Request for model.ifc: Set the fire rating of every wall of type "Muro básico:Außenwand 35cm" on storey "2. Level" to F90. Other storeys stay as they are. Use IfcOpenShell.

First a look at what the model holds.

```python
import ifcopenshell
import ifcopenshell.util.element

model = ifcopenshell.open("model.ifc")
print(model.schema)
storey = next(s for s in model.by_type("IfcBuildingStorey") if s.Name == "2. Level")
walls = [e for e in ifcopenshell.util.element.get_decomposition(storey) if e.is_a("IfcWall")]
seen = {}
for e in walls:
    element_type = ifcopenshell.util.element.get_type(e)
    key = (element_type.Name if element_type != e and element_type else None, ifcopenshell.util.element.get_pset(e, "Pset_WallCommon", "FireRating"))
    seen[key] = seen.get(key, 0) + 1
for (name, value), count in sorted(seen.items(), key=str):
    print(count, "x", name, "|", value)
```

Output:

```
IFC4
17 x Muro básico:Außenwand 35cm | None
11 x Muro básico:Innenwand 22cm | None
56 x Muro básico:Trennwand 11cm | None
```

```python
import ifcopenshell
import ifcopenshell.api.pset
import ifcopenshell.util.element

model = ifcopenshell.open("model.ifc")

storey = next(s for s in model.by_type("IfcBuildingStorey") if s.Name == "2. Level")
walls = [e for e in ifcopenshell.util.element.get_decomposition(storey) if e.is_a("IfcWall")]

count = 0
for e in walls:
    element_type = ifcopenshell.util.element.get_type(e)
    if element_type in (None, e) or element_type.Name != "Muro básico:Außenwand 35cm":
        continue
    # add_pset returns the element's existing set when there is one.
    pset = ifcopenshell.api.pset.add_pset(model, product=e, name="Pset_WallCommon")
    ifcopenshell.api.pset.edit_pset(model, pset=pset, properties={"FireRating": "F90"})
    count += 1

print(count, "walls updated")

model.write("model_v2.ifc")
```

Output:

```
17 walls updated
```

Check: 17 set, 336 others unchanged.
